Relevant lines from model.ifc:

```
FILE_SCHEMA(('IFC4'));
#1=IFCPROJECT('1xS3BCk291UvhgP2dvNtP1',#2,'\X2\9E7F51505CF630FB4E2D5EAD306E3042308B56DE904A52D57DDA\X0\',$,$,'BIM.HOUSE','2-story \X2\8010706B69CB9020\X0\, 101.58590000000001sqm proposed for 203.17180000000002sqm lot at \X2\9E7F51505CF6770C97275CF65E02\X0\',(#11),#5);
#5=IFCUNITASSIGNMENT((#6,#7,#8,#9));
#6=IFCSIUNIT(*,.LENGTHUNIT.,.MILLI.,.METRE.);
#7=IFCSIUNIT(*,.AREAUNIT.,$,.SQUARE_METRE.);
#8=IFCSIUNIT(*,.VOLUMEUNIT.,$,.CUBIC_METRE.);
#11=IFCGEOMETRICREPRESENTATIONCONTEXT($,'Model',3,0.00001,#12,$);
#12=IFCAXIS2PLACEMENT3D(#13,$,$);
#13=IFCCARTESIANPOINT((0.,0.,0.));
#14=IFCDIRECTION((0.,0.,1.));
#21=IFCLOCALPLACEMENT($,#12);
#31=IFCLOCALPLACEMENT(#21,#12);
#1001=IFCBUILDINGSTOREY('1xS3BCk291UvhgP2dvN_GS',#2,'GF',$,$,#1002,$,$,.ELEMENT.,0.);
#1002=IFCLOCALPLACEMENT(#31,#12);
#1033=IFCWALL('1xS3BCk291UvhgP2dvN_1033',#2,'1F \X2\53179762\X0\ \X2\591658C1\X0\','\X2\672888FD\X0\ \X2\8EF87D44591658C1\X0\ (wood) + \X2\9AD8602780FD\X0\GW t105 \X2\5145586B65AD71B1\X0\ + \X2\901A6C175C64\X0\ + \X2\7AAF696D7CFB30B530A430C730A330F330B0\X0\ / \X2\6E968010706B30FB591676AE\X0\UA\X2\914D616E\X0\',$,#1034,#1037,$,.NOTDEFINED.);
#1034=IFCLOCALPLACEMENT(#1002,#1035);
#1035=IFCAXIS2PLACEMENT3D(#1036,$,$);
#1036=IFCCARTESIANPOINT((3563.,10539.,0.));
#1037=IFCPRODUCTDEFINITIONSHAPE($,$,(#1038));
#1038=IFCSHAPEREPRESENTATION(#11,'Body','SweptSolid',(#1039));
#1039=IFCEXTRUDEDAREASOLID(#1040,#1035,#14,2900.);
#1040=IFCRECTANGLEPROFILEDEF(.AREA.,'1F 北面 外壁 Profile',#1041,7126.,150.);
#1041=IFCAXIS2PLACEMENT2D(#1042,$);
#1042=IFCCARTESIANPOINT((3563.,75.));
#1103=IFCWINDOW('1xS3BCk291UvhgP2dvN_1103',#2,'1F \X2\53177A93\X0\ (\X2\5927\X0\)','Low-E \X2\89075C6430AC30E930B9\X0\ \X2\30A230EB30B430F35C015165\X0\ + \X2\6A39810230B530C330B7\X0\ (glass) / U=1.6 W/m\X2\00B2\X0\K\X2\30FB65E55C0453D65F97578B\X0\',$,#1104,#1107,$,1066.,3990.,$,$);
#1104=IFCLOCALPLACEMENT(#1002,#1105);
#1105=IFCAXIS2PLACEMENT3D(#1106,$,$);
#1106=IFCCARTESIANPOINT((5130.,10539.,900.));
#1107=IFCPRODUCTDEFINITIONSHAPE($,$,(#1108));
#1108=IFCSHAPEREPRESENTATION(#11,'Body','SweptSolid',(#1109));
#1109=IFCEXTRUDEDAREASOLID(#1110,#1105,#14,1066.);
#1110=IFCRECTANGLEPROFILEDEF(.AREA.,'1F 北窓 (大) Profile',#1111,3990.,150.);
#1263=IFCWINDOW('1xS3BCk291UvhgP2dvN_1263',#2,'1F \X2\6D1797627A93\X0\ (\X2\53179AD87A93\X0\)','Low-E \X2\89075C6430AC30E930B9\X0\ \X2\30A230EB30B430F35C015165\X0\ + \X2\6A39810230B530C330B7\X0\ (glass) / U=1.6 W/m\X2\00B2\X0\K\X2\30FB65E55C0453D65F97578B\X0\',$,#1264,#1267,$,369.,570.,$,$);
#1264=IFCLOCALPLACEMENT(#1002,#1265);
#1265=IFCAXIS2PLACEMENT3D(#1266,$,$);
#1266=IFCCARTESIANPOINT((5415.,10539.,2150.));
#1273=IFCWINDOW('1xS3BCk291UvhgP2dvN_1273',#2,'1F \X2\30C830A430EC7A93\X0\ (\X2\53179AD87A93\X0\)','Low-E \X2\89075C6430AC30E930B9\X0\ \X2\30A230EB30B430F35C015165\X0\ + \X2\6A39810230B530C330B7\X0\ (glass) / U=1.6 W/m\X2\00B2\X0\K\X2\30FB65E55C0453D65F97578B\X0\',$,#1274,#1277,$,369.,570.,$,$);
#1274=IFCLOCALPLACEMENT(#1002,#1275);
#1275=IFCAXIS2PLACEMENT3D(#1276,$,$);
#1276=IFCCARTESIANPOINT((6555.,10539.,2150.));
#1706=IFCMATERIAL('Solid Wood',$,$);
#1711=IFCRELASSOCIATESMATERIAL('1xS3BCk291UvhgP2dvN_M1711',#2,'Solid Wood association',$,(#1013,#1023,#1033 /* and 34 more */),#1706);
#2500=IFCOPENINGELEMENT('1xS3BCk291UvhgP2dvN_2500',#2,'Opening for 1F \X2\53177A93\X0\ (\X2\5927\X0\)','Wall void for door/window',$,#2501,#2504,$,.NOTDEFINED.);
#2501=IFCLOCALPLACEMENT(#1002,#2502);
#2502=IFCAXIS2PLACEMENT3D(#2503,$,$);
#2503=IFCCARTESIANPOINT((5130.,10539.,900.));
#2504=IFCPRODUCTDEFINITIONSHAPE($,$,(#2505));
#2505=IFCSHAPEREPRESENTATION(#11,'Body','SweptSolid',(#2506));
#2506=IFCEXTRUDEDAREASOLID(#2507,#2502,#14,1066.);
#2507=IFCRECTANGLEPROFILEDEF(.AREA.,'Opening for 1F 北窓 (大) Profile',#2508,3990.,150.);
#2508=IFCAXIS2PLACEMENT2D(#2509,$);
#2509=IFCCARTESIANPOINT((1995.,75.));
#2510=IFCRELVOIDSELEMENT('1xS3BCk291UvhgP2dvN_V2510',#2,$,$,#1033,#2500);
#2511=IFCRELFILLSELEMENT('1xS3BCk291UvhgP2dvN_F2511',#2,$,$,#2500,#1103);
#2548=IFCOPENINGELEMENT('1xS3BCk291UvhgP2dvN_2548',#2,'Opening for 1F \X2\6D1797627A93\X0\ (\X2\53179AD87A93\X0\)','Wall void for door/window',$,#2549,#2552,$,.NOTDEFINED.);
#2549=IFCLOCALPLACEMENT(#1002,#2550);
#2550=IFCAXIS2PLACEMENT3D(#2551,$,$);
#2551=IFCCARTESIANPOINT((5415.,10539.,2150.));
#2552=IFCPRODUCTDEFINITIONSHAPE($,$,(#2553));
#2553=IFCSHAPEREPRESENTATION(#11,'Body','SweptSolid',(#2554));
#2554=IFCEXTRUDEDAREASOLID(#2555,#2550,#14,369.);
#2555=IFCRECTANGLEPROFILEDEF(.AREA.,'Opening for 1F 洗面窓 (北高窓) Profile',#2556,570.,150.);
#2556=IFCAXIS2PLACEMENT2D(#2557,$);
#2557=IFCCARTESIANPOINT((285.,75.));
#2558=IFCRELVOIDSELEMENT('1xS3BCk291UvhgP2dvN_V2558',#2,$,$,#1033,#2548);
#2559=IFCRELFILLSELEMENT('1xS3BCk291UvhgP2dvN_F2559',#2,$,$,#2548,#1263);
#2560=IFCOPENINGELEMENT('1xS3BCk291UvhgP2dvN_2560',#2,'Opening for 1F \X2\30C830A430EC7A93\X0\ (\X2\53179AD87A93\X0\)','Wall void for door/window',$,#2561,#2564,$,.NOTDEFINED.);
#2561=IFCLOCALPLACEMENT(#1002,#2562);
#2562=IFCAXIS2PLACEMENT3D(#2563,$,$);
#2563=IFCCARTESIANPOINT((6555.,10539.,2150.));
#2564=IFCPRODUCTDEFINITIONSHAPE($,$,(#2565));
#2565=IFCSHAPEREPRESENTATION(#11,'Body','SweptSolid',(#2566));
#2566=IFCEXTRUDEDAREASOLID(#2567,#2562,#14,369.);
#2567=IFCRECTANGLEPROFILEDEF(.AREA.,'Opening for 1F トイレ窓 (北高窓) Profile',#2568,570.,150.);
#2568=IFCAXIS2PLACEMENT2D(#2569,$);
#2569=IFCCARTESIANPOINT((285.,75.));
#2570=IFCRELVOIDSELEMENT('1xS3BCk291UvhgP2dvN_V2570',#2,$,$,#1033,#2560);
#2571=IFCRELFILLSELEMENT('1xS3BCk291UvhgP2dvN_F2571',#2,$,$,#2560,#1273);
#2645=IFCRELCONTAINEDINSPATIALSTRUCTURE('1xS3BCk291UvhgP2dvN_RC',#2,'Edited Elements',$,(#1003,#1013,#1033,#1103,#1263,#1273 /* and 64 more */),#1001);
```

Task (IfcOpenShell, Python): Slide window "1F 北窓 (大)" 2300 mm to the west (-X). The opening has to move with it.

```python
import ifcopenshell
import ifcopenshell.api.geometry
import ifcopenshell.util.placement

model = ifcopenshell.open("model.ifc")

window = model.by_guid("1xS3BCk291UvhgP2dvN_1103")
opening = window.FillsVoids[0].RelatingOpeningElement
wall = opening.VoidsElements[0].RelatingBuildingElement

wall_matrix = ifcopenshell.util.placement.get_local_placement(wall.ObjectPlacement)
shift = wall_matrix[:3, 0] * -2300.0
before = ifcopenshell.util.placement.get_local_placement(window.ObjectPlacement)[:3, 3].copy()

# The window is not placed relative to its opening, so move both.
for product in (opening, window):
    matrix = ifcopenshell.util.placement.get_local_placement(product.ObjectPlacement)
    matrix[:3, 3] += shift
    ifcopenshell.api.geometry.edit_object_placement(model, product=product, matrix=matrix, is_si=False)

after = ifcopenshell.util.placement.get_local_placement(window.ObjectPlacement)[:3, 3]
print("window moved by", (after - before).round(3) + 0.0)

model.write("model_edited.ifc")
```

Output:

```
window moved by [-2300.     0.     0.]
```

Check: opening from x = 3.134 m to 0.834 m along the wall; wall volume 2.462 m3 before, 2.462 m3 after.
